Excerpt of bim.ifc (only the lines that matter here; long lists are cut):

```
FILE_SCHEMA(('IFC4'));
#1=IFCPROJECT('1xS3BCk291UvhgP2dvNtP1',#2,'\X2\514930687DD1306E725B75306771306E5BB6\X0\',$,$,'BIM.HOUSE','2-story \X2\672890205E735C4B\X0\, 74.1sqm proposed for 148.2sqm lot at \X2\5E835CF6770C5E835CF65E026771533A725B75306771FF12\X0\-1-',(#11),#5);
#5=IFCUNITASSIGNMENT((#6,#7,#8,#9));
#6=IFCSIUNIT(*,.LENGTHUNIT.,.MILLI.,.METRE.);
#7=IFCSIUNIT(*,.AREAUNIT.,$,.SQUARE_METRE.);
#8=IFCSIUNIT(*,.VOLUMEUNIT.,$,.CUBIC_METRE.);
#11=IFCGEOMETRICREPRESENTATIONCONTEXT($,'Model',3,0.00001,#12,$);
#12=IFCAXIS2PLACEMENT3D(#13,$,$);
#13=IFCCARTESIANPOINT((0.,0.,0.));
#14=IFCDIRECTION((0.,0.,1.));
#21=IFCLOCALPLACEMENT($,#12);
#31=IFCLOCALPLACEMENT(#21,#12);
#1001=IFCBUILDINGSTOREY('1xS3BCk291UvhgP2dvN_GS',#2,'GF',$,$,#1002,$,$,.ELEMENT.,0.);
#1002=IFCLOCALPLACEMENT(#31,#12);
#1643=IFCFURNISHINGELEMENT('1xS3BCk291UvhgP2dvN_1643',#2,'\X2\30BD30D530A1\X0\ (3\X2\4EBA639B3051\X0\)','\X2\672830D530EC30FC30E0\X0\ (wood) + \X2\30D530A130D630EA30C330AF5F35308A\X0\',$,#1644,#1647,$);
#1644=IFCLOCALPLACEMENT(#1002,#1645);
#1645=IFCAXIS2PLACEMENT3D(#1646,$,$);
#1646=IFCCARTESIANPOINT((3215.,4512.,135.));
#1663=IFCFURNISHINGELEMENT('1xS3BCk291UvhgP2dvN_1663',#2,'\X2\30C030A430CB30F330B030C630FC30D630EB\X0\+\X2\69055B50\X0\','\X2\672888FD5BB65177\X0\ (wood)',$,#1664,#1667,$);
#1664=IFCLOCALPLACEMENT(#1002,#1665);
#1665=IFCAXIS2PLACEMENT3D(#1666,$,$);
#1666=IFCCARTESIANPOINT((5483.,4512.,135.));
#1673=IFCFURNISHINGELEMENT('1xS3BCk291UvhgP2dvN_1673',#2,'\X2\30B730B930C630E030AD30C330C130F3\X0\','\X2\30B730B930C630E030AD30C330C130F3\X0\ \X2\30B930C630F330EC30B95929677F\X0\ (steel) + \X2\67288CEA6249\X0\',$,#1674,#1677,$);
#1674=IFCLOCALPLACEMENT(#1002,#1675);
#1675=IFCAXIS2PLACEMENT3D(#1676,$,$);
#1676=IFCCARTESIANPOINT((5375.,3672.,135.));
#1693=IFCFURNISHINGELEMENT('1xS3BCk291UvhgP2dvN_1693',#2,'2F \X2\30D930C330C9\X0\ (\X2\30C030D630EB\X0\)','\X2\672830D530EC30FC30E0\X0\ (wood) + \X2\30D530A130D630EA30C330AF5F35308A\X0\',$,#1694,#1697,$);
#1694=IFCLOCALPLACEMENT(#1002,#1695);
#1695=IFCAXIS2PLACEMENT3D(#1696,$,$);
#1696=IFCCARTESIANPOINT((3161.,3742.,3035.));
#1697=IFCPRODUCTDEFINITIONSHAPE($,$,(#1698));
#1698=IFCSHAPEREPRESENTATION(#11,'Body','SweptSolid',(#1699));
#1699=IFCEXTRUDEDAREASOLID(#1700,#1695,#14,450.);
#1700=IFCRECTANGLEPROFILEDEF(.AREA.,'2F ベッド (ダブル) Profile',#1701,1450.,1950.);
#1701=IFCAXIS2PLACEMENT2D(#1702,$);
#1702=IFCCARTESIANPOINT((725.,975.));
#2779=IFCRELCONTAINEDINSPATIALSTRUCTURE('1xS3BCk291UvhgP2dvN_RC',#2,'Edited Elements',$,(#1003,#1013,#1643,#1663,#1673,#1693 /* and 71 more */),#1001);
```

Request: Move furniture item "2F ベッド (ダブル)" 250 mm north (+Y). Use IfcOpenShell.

```python
import ifcopenshell
import ifcopenshell.api.geometry
import ifcopenshell.util.placement

model = ifcopenshell.open("bim.ifc")

item = model.by_guid("1xS3BCk291UvhgP2dvN_1693")
matrix = ifcopenshell.util.placement.get_local_placement(item.ObjectPlacement)
matrix[1, 3] += 250.0
ifcopenshell.api.geometry.edit_object_placement(model, product=item, matrix=matrix, is_si=False)

print(ifcopenshell.util.placement.get_local_placement(item.ObjectPlacement).round(3) + 0.0)

model.write("bim_rev.ifc")
```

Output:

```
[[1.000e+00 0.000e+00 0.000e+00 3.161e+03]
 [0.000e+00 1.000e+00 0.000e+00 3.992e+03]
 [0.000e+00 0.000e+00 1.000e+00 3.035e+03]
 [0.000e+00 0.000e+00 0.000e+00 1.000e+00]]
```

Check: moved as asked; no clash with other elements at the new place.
